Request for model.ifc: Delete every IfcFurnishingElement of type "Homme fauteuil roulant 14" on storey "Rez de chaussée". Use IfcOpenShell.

First a look at what the model holds.

```python
import ifcopenshell
import ifcopenshell.util.element

model = ifcopenshell.open("model.ifc")
print(model.schema)
storey = next(s for s in model.by_type("IfcBuildingStorey") if s.Name == "Rez de chaussée")
furniture = [e for e in ifcopenshell.util.element.get_decomposition(storey) if e.is_a("IfcFurnishingElement")]
seen = {}
for e in furniture:
    element_type = ifcopenshell.util.element.get_type(e)
    name = element_type.Name if element_type not in (None, e) else None
    seen[name] = seen.get(name, 0) + 1
for name, count in sorted(seen.items(), key=str):
    print(count, "x", name)
```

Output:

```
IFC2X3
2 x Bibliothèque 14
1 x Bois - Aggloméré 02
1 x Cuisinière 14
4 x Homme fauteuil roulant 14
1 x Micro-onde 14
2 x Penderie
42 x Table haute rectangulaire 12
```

```python
import ifcopenshell
import ifcopenshell.api.root
import ifcopenshell.util.element

model = ifcopenshell.open("model.ifc")

storey = next(s for s in model.by_type("IfcBuildingStorey") if s.Name == "Rez de chaussée")
furniture = [e for e in ifcopenshell.util.element.get_decomposition(storey) if e.is_a("IfcFurnishingElement")]
targets = [e for e in furniture if (t := ifcopenshell.util.element.get_type(e)) not in (None, e) and t.Name == "Homme fauteuil roulant 14"]

for e in targets:
    ifcopenshell.api.root.remove_product(model, product=e)
print(len(targets), "removed")

model.write("model_rev.ifc")
```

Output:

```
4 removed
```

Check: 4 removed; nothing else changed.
